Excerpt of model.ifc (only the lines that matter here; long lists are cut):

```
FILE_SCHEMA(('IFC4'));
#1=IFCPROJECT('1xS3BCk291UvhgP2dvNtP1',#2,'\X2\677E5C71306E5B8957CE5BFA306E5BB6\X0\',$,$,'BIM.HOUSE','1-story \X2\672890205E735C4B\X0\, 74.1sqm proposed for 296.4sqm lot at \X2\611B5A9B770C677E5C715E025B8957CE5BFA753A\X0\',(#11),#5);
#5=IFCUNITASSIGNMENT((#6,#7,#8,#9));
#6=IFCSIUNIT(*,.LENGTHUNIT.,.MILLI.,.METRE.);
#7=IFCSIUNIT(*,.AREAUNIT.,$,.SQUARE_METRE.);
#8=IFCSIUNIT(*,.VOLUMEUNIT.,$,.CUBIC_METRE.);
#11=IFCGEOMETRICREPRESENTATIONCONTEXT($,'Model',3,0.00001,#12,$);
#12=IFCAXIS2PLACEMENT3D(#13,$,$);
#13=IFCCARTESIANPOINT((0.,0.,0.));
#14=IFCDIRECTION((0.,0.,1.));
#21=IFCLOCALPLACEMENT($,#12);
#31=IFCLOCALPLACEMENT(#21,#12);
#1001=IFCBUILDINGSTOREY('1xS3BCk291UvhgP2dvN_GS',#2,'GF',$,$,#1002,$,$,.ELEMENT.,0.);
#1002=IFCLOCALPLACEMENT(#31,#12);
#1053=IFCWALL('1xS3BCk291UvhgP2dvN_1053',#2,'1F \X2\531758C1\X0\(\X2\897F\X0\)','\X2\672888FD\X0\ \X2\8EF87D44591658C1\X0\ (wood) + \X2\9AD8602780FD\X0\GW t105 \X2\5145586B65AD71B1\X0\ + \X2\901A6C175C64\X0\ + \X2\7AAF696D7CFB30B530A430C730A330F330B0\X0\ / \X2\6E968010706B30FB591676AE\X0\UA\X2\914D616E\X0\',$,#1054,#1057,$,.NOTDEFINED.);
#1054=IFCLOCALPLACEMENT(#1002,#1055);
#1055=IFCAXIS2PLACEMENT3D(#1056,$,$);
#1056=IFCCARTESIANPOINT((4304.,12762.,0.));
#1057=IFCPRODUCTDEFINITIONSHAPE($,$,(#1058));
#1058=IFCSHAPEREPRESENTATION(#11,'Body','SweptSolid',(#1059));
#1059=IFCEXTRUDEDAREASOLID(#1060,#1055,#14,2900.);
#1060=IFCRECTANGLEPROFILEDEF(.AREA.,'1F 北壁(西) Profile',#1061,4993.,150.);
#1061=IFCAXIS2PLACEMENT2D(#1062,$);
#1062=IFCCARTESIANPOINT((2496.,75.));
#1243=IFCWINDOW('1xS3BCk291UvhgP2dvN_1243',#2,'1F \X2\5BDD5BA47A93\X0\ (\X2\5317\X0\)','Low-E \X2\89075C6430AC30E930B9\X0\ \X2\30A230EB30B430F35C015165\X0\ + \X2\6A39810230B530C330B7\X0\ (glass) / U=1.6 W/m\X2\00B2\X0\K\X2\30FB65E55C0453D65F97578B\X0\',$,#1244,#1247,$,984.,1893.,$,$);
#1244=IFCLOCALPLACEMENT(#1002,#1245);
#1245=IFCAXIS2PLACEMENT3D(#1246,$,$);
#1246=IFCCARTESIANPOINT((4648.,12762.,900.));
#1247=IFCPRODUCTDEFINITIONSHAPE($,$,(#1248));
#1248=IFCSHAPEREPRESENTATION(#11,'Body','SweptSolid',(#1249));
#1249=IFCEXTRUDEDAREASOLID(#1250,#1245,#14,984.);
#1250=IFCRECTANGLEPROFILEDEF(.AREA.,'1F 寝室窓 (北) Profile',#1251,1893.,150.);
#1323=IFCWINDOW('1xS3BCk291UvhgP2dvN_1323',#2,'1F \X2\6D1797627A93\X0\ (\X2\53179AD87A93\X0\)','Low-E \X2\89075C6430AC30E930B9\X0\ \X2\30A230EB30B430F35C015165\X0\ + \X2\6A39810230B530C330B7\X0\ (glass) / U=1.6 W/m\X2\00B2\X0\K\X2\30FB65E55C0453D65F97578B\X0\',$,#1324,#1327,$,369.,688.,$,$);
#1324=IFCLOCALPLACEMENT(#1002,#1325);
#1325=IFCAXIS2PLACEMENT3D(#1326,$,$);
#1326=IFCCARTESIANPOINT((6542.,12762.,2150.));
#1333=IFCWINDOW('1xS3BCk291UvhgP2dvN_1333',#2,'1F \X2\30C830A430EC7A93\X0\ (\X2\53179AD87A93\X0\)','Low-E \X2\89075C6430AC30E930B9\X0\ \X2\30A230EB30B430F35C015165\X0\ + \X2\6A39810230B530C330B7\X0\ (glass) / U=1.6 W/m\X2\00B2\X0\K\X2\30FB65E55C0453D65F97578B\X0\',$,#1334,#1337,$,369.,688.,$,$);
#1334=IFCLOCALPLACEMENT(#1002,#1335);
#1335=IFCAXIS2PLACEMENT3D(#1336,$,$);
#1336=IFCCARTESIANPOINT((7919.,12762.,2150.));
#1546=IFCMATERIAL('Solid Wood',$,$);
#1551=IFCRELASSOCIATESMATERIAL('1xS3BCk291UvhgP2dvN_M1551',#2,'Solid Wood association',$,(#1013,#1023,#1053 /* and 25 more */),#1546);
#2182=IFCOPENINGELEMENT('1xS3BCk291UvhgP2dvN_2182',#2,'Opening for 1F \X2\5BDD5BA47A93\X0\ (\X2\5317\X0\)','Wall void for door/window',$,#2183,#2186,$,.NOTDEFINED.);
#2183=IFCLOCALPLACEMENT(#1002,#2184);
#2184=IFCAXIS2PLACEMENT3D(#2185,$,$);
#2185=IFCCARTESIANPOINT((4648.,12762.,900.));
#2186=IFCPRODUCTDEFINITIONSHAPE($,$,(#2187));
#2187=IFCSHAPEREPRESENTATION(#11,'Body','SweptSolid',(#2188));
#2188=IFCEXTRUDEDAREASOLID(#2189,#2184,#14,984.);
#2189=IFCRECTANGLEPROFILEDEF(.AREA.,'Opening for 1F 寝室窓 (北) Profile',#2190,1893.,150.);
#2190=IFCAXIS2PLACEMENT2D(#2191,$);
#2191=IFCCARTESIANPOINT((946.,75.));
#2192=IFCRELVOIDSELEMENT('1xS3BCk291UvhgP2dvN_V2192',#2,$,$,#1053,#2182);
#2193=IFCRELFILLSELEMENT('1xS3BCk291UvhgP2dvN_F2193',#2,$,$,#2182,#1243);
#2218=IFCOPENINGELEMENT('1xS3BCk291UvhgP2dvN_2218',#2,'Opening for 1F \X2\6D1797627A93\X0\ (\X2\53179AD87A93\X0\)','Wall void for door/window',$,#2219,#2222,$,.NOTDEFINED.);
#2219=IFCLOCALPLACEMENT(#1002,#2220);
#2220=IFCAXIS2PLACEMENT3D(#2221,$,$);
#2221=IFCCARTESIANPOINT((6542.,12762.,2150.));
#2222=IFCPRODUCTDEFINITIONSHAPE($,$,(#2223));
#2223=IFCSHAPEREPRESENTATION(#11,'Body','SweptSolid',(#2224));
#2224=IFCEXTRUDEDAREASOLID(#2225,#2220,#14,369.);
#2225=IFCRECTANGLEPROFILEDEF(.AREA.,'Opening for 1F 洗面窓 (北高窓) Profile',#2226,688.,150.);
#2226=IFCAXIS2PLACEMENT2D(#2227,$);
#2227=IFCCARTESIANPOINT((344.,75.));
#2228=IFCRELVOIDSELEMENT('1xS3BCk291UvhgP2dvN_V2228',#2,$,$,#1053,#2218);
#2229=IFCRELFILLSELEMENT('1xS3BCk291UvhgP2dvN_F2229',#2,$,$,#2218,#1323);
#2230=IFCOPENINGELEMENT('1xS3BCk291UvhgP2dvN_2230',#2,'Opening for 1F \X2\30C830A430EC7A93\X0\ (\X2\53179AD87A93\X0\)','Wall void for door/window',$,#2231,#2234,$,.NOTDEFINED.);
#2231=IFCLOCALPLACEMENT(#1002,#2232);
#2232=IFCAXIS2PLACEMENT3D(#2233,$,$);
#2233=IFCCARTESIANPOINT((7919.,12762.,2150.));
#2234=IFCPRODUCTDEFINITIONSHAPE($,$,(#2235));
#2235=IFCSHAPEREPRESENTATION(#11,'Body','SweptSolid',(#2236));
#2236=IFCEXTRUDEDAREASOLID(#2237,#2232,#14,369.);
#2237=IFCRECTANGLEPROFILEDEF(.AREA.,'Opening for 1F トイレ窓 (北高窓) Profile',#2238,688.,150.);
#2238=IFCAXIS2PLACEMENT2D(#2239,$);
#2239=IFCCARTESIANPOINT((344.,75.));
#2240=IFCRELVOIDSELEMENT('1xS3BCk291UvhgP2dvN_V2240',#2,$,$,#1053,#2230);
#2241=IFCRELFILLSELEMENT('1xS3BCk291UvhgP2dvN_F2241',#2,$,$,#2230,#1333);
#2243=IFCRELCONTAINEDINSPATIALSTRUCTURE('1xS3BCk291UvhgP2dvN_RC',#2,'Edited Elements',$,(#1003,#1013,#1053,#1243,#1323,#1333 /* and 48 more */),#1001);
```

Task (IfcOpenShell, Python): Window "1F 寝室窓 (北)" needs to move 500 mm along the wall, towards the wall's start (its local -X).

```python
import ifcopenshell
import ifcopenshell.api.geometry
import ifcopenshell.util.placement

model = ifcopenshell.open("model.ifc")

window = model.by_guid("1xS3BCk291UvhgP2dvN_1243")
opening = window.FillsVoids[0].RelatingOpeningElement
wall = opening.VoidsElements[0].RelatingBuildingElement

wall_matrix = ifcopenshell.util.placement.get_local_placement(wall.ObjectPlacement)
shift = wall_matrix[:3, 0] * -500.0
before = ifcopenshell.util.placement.get_local_placement(window.ObjectPlacement)[:3, 3].copy()

# The window is not placed relative to its opening, so move both.
for product in (opening, window):
    matrix = ifcopenshell.util.placement.get_local_placement(product.ObjectPlacement)
    matrix[:3, 3] += shift
    ifcopenshell.api.geometry.edit_object_placement(model, product=product, matrix=matrix, is_si=False)

after = ifcopenshell.util.placement.get_local_placement(window.ObjectPlacement)[:3, 3]
print("window moved by", (after - before).round(3) + 0.0)

model.write("model_edited.ifc")
```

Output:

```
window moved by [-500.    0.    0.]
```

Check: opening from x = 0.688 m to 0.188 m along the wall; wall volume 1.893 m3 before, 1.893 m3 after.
